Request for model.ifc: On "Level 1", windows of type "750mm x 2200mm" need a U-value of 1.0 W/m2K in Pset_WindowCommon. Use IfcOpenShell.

First a look at what the model holds.

```python
import ifcopenshell
import ifcopenshell.util.element

model = ifcopenshell.open("model.ifc")
print(model.schema)
storey = next(s for s in model.by_type("IfcBuildingStorey") if s.Name == "Level 1")
windows = [e for e in ifcopenshell.util.element.get_decomposition(storey) if e.is_a("IfcWindow")]
seen = {}
for e in windows:
    element_type = ifcopenshell.util.element.get_type(e)
    key = (element_type.Name if element_type != e and element_type else None, ifcopenshell.util.element.get_pset(e, "Pset_WindowCommon", "ThermalTransmittance"))
    seen[key] = seen.get(key, 0) + 1
for (name, value), count in sorted(seen.items(), key=str):
    print(count, "x", name, "|", value)
```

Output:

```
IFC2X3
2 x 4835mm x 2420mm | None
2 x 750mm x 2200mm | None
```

```python
import ifcopenshell
import ifcopenshell.api.pset
import ifcopenshell.util.element

model = ifcopenshell.open("model.ifc")

storey = next(s for s in model.by_type("IfcBuildingStorey") if s.Name == "Level 1")
windows = [e for e in ifcopenshell.util.element.get_decomposition(storey) if e.is_a("IfcWindow")]

count = 0
for e in windows:
    element_type = ifcopenshell.util.element.get_type(e)
    if element_type in (None, e) or element_type.Name != "750mm x 2200mm":
        continue
    # add_pset returns the element's existing set when there is one.
    pset = ifcopenshell.api.pset.add_pset(model, product=e, name="Pset_WindowCommon")
    ifcopenshell.api.pset.edit_pset(model, pset=pset, properties={"ThermalTransmittance": 1.0})
    count += 1

print(count, "windows updated")

model.write("model-out.ifc")
```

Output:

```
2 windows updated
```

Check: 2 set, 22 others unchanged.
